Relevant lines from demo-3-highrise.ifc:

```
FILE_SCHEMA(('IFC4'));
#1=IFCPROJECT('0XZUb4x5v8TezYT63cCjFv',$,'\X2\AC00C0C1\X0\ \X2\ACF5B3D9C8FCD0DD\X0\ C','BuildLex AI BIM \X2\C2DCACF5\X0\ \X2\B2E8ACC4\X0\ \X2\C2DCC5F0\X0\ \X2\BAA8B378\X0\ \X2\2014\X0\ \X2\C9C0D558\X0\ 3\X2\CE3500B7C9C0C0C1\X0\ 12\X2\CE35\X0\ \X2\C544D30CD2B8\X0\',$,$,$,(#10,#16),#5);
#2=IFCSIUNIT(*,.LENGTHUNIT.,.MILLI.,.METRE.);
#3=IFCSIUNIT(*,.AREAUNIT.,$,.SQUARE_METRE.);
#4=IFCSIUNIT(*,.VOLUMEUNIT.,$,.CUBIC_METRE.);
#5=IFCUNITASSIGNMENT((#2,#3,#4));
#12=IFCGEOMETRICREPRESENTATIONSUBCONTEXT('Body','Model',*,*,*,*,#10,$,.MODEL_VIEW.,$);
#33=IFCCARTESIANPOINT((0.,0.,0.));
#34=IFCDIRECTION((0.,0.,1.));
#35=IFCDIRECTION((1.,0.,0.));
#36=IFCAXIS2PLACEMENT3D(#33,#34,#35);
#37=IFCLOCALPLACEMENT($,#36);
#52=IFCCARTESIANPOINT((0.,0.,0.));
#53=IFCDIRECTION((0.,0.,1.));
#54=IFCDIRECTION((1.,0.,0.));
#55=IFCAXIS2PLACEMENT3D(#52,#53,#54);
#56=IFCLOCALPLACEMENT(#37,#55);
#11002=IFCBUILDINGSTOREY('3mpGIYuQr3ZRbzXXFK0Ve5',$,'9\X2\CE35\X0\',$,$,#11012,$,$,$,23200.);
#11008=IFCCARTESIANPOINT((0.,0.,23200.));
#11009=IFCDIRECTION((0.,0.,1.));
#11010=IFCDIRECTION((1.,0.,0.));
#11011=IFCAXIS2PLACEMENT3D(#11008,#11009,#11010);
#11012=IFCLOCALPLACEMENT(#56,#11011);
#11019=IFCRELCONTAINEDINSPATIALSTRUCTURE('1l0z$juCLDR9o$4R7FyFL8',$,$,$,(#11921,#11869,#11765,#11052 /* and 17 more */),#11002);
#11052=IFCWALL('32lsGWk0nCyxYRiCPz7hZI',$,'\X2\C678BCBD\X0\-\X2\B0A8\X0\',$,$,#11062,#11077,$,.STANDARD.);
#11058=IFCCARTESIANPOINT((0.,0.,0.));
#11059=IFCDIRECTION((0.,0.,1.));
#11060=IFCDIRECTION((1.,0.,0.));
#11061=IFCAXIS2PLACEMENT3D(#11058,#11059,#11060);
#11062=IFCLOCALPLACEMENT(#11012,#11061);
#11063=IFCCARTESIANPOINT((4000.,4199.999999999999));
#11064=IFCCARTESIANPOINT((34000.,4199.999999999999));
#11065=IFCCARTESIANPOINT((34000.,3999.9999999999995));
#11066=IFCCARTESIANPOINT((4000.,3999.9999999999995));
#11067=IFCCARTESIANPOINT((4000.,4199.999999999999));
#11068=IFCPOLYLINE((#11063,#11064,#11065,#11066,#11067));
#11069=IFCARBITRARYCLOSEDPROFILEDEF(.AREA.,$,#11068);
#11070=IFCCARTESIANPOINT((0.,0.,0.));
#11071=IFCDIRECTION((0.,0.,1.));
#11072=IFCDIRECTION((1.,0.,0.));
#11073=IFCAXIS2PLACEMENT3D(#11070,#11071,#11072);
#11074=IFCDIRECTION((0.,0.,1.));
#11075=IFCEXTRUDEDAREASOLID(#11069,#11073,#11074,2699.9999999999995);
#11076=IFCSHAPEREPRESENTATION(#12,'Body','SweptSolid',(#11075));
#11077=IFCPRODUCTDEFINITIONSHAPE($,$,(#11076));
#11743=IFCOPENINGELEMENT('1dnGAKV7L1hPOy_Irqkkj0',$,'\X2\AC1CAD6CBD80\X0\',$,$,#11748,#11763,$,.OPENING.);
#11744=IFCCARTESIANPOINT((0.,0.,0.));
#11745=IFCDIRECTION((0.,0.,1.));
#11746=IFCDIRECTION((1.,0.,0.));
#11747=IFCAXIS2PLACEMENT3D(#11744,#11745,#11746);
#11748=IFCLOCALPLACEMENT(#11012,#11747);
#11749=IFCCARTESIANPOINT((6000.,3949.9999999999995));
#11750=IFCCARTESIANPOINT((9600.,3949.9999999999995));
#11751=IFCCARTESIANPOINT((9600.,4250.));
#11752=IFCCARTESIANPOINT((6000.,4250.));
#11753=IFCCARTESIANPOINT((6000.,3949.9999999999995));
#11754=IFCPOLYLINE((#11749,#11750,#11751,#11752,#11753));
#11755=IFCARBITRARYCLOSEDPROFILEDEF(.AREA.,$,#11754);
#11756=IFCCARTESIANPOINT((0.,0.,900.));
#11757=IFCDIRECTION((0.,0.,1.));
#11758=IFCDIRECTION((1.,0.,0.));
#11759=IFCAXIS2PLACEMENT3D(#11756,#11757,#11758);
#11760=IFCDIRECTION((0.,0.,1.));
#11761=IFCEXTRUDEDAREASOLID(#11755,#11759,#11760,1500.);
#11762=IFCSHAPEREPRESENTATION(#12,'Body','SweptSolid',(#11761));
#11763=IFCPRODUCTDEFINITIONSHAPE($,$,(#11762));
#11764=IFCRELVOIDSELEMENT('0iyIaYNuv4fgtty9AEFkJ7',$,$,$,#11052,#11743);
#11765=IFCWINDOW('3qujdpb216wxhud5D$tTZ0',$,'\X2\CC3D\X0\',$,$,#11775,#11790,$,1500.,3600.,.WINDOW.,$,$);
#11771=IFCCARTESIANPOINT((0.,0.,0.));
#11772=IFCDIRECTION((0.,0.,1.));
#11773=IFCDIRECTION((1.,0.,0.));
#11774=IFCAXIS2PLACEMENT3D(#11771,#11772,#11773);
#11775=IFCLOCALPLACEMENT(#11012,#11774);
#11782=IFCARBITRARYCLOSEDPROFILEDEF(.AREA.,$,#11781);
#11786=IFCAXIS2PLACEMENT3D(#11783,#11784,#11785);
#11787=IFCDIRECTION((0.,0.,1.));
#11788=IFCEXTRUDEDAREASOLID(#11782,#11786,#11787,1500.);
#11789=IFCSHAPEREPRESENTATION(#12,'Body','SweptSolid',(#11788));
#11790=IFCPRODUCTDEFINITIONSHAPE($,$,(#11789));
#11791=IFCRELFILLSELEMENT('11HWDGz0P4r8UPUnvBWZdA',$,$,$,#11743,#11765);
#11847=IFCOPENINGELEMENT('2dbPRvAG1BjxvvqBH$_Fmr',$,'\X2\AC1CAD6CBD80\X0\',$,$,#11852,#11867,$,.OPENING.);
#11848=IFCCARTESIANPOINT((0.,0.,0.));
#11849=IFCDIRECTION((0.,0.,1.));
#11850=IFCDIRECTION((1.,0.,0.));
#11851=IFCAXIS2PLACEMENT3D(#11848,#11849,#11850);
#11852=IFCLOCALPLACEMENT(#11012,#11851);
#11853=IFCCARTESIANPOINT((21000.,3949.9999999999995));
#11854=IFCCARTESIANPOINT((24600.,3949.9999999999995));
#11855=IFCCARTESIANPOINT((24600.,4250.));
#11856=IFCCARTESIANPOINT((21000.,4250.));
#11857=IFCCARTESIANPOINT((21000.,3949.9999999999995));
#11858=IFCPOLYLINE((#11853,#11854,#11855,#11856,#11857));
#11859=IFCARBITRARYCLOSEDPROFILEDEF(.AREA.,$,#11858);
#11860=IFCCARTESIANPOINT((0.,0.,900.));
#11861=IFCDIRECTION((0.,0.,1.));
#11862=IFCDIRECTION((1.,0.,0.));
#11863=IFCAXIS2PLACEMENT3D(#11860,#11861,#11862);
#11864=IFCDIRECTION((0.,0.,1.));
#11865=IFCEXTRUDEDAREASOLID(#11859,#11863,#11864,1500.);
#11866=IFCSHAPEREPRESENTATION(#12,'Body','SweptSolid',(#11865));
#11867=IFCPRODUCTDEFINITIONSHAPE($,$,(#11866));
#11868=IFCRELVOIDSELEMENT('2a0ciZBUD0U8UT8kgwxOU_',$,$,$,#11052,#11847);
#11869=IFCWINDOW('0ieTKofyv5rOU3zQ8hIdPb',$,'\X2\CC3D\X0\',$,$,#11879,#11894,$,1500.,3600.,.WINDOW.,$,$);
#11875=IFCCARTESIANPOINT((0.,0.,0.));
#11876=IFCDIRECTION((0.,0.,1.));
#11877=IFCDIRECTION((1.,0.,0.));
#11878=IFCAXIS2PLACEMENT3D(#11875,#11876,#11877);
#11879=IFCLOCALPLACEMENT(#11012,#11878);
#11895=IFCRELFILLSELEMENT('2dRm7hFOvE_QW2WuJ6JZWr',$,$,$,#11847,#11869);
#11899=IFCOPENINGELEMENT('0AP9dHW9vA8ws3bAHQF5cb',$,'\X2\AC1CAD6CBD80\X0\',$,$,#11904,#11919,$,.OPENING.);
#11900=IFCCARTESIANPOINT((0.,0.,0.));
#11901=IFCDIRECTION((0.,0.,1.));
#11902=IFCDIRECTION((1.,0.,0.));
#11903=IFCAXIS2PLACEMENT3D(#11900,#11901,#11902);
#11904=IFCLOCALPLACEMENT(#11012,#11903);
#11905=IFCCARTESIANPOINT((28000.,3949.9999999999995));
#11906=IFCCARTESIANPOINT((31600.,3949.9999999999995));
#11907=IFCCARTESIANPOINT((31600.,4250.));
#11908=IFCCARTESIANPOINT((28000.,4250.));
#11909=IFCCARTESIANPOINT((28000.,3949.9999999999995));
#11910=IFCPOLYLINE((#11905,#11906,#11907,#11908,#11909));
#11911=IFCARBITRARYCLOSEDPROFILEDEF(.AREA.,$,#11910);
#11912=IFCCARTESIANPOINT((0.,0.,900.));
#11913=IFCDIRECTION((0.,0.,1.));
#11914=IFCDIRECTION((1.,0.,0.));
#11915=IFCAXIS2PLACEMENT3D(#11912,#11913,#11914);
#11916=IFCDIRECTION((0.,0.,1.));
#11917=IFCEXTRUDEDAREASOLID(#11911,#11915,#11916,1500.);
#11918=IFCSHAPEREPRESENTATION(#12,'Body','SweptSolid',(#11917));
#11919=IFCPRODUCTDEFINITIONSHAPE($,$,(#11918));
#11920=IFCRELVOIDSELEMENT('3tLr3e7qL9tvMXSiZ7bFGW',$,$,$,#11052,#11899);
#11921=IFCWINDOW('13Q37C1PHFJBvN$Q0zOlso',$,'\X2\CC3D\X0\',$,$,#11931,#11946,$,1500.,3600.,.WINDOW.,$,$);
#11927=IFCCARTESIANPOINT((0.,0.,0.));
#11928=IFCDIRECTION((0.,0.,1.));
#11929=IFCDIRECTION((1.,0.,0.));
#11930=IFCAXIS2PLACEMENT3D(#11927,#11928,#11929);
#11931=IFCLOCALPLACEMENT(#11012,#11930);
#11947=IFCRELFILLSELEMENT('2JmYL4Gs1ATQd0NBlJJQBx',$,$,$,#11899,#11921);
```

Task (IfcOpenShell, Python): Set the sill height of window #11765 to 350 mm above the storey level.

```python
import numpy as np
import ifcopenshell
import ifcopenshell.api.geometry
import ifcopenshell.geom
import ifcopenshell.util.element
import ifcopenshell.util.placement
import ifcopenshell.util.shape
import ifcopenshell.util.unit

model = ifcopenshell.open("demo-3-highrise.ifc")
unit_scale = ifcopenshell.util.unit.calculate_unit_scale(model)

window = model.by_guid("3qujdpb216wxhud5D$tTZ0")
opening = window.FillsVoids[0].RelatingOpeningElement
storey = ifcopenshell.util.element.get_container(window, ifc_class="IfcBuildingStorey")
level = ifcopenshell.util.placement.get_local_placement(storey.ObjectPlacement)[2, 3]

# The opening's origin need not be at the sill, so measure its lowest point.
shape = ifcopenshell.geom.create_shape(ifcopenshell.geom.settings(), opening)
bottom = ifcopenshell.util.shape.get_shape_bottom_elevation(shape, shape.geometry) / unit_scale
dz = level + 0.35 / unit_scale - bottom

shift = np.array([0.0, 0.0, dz])
# The window is not placed relative to its opening, so move both.
for product in (opening, window):
    matrix = ifcopenshell.util.placement.get_local_placement(product.ObjectPlacement)
    matrix[:3, 3] += shift
    ifcopenshell.api.geometry.edit_object_placement(model, product=product, matrix=matrix, is_si=False)

print(f"moved by {dz * unit_scale:+.3f} m")

model.write("demo-3-highrise-out.ifc")
```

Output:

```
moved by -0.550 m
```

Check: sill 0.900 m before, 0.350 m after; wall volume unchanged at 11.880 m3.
